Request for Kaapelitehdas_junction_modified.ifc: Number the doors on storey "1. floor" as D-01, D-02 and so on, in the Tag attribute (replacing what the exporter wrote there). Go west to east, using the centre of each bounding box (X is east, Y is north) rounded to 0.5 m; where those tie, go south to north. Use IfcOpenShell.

First a look at what the model holds.

```python
import ifcopenshell
import ifcopenshell.util.element
import ifcopenshell.util.placement

model = ifcopenshell.open("Kaapelitehdas_junction_modified.ifc")
print(model.schema)
storey = next(s for s in model.by_type("IfcBuildingStorey") if s.Name == "1. floor")
doors = [e for e in ifcopenshell.util.element.get_decomposition(storey) if e.is_a("IfcDoor")]
for e in sorted(doors, key=lambda e: e.id()):
    origin = ifcopenshell.util.placement.get_local_placement(e.ObjectPlacement)[:3, 3]
    print(e.id(), e.Tag, e.Name, origin.round(2) + 0.0, sep=" | ")
```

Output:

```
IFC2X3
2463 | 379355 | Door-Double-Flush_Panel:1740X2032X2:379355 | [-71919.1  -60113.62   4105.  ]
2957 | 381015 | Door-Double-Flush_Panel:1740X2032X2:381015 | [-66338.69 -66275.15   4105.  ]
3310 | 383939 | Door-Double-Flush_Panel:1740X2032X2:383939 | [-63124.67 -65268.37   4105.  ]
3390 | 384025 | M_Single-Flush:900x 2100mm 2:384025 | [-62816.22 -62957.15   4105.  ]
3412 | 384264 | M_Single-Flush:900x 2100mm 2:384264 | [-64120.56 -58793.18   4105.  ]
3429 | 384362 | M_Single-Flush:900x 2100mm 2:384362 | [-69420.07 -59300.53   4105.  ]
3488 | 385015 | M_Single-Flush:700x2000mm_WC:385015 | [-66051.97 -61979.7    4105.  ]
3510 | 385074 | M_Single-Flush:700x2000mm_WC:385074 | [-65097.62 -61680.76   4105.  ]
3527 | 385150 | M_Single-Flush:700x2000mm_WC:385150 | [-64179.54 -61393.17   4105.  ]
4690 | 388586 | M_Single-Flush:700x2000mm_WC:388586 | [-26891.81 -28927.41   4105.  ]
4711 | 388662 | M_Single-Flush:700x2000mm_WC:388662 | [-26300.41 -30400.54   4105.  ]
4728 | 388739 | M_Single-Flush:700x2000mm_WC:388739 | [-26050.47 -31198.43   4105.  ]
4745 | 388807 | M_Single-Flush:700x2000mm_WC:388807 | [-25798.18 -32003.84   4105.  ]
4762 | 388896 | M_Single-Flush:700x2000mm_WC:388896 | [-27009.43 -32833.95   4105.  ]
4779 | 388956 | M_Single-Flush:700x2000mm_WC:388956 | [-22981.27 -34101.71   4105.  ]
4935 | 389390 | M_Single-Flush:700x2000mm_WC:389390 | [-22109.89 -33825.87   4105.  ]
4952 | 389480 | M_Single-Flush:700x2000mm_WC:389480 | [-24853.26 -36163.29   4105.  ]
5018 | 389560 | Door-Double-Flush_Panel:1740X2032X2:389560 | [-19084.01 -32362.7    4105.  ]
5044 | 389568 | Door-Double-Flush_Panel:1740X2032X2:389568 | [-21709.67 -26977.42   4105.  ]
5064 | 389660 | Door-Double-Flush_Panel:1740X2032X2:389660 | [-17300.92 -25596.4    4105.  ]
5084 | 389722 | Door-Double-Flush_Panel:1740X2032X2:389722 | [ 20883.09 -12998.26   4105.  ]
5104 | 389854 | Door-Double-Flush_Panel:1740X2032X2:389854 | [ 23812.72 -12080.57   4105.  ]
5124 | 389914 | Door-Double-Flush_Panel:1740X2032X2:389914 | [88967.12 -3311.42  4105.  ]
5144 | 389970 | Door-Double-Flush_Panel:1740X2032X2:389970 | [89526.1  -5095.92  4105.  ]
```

```python
import ifcopenshell
import ifcopenshell.geom
import ifcopenshell.util.element
import ifcopenshell.util.shape

model = ifcopenshell.open("Kaapelitehdas_junction_modified.ifc")
settings = ifcopenshell.geom.settings()
settings.set("use-world-coords", True)


def centre(element):
    shape = ifcopenshell.geom.create_shape(settings, element)
    return ifcopenshell.util.shape.get_bbox_centroid(shape.geometry)


storey = next(s for s in model.by_type("IfcBuildingStorey") if s.Name == "1. floor")
doors = [e for e in ifcopenshell.util.element.get_decomposition(storey) if e.is_a("IfcDoor")]

# Insertion points can sit at a corner or the storey origin, so sort by the geometry (in metres).
centres = {e: centre(e) for e in doors}
doors.sort(key=lambda e: (round(centres[e][0] / 0.5), centres[e][1]))

for i, e in enumerate(doors, start=1):
    number = f"D-{i:02d}"
    e.Tag = number
    print(e.id(), number)

model.write("Kaapelitehdas_junction_modified_v2.ifc")
```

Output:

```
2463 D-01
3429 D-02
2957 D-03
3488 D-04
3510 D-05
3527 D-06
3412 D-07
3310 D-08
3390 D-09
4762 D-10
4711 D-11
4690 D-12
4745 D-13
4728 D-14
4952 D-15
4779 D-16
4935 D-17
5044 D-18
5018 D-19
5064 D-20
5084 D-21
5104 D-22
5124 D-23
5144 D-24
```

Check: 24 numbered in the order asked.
